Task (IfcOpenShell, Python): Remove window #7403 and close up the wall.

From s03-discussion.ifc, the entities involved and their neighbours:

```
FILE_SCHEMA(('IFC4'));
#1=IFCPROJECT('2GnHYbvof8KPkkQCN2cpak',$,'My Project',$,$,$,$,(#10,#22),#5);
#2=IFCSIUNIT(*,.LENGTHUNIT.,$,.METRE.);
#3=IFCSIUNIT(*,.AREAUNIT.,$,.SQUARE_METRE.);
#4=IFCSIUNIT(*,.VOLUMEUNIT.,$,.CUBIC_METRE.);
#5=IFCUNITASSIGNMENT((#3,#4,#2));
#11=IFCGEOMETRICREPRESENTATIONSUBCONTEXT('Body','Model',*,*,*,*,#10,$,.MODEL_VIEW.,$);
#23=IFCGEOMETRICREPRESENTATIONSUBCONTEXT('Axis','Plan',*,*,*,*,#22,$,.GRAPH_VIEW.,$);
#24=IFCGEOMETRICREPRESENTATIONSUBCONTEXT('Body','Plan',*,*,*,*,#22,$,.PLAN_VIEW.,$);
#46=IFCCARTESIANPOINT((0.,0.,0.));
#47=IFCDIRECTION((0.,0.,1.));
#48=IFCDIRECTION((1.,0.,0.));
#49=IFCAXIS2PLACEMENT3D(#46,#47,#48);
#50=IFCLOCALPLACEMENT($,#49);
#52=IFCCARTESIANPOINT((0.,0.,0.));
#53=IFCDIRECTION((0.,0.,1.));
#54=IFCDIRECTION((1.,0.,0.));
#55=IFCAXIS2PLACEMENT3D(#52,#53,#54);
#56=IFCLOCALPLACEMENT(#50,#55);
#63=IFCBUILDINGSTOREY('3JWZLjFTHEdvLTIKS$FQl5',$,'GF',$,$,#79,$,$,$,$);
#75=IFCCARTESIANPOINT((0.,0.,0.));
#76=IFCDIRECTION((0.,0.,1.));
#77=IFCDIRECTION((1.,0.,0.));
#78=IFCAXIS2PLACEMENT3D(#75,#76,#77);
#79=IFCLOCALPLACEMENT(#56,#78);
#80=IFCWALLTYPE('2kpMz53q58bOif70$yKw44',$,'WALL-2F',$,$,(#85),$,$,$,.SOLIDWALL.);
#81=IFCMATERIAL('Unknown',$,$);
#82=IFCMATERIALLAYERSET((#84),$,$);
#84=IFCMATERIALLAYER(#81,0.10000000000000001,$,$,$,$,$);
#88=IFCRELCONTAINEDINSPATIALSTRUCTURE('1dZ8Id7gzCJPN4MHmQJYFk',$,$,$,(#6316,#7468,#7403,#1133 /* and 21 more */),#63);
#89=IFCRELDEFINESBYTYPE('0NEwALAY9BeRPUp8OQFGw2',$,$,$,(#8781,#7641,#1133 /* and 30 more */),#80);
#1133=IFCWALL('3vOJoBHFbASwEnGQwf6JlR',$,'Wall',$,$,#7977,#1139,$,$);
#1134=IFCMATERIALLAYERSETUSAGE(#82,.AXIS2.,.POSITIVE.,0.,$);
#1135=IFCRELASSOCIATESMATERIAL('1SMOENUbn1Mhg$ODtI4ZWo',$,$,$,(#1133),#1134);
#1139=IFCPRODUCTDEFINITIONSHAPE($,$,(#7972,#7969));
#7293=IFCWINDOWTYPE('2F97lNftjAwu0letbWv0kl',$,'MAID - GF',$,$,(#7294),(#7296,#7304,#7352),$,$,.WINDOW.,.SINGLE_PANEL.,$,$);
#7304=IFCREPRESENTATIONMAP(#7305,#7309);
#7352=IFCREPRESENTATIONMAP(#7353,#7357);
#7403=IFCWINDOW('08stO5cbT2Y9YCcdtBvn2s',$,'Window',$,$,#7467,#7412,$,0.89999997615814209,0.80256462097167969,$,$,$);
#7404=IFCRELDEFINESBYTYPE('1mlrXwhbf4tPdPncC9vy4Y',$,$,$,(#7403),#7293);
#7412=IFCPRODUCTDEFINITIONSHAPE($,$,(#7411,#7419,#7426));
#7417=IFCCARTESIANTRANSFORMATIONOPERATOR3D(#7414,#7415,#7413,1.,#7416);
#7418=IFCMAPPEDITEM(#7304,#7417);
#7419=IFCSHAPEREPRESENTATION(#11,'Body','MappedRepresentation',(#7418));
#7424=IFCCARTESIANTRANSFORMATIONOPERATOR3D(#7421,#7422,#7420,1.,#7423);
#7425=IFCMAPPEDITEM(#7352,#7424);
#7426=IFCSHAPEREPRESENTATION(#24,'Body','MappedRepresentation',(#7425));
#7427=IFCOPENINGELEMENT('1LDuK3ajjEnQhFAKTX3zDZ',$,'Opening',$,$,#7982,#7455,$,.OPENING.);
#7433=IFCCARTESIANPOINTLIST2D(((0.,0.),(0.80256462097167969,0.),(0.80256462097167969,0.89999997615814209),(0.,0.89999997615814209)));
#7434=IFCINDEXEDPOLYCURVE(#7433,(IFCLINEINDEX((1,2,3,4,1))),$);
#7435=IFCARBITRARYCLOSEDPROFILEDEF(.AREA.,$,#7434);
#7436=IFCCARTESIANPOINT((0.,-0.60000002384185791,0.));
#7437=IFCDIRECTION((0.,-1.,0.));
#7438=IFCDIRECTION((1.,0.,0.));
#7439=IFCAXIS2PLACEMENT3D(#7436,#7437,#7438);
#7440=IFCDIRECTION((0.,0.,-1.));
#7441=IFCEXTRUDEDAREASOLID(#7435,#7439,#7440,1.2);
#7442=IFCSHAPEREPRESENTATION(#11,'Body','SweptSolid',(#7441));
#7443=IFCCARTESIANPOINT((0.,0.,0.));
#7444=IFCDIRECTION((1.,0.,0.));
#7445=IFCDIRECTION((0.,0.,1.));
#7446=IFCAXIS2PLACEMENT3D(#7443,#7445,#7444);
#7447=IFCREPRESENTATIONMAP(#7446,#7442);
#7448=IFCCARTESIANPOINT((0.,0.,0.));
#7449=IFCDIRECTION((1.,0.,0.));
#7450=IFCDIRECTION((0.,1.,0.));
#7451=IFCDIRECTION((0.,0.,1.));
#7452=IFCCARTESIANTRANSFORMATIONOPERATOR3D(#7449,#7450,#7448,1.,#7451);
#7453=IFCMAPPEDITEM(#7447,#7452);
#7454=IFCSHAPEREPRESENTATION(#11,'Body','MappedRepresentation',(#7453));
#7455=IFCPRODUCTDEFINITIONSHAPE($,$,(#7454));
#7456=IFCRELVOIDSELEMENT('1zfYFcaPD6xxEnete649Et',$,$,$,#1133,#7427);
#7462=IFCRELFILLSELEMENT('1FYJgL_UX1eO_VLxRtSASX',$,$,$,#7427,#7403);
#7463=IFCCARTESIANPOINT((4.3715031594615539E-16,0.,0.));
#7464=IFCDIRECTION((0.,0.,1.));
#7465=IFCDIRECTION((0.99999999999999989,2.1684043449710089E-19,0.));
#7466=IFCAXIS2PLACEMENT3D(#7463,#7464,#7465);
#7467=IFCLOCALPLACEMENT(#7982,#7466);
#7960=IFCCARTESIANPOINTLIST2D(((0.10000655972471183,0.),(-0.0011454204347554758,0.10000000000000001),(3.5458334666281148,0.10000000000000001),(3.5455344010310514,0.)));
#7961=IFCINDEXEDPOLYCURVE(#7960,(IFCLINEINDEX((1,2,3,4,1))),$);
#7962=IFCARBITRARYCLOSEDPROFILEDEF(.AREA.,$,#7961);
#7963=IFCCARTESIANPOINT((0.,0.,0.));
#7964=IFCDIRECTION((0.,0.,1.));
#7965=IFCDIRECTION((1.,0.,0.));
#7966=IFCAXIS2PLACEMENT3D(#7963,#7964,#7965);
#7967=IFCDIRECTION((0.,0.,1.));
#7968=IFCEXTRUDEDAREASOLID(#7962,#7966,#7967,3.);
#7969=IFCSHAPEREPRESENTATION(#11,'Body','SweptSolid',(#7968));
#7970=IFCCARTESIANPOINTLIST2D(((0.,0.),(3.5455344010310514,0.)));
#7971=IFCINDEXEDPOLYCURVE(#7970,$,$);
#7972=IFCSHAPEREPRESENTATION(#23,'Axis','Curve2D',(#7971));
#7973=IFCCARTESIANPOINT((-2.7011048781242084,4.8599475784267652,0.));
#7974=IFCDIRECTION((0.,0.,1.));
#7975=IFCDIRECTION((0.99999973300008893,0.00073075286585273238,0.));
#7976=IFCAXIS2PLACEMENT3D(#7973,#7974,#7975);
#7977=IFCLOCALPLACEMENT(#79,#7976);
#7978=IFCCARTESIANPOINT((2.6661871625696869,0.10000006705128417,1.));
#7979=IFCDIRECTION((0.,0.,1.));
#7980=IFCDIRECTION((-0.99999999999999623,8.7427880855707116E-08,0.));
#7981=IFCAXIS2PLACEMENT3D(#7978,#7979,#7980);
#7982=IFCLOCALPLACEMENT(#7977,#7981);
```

```python
import ifcopenshell
import ifcopenshell.api.feature
import ifcopenshell.api.root
import ifcopenshell.geom
import ifcopenshell.util.shape

model = ifcopenshell.open("s03-discussion.ifc")
settings = ifcopenshell.geom.settings()


def volume(element):
    """Net volume in cubic metres, openings subtracted."""
    shape = ifcopenshell.geom.create_shape(settings, element)
    return ifcopenshell.util.shape.get_volume(shape.geometry)


window = model.by_guid("08stO5cbT2Y9YCcdtBvn2s")
opening = window.FillsVoids[0].RelatingOpeningElement
wall = opening.VoidsElements[0].RelatingBuildingElement
before = volume(wall)

ifcopenshell.api.root.remove_product(model, product=window)
ifcopenshell.api.feature.remove_feature(model, feature=opening)

after = volume(wall)

print(f"wall volume {before:.3f} -> {after:.3f} m3")

model.write("s03-discussion-out.ifc")
```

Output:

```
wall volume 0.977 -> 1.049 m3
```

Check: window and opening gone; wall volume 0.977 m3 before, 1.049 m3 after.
